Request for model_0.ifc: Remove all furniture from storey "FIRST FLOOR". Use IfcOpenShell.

First a look at what the model holds.

```python
import ifcopenshell
import ifcopenshell.util.element

model = ifcopenshell.open("model_0.ifc")
print(model.schema)
storey = next(s for s in model.by_type("IfcBuildingStorey") if s.Name == "FIRST FLOOR")
furniture = [e for e in ifcopenshell.util.element.get_decomposition(storey) if e.is_a("IfcFurnishingElement")]
seen = {}
for e in furniture:
    element_type = ifcopenshell.util.element.get_type(e)
    name = element_type.Name if element_type not in (None, e) else None
    seen[name] = seen.get(name, 0) + 1
for name, count in sorted(seen.items(), key=str):
    print(count, "x", name)
```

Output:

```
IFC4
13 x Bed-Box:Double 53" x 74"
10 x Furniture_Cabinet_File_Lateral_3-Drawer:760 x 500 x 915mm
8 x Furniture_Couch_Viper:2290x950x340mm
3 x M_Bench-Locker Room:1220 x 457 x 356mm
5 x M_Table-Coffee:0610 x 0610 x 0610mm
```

```python
import ifcopenshell
import ifcopenshell.api.root
import ifcopenshell.util.element

model = ifcopenshell.open("model_0.ifc")

storey = next(s for s in model.by_type("IfcBuildingStorey") if s.Name == "FIRST FLOOR")
furniture = [e for e in ifcopenshell.util.element.get_decomposition(storey) if e.is_a("IfcFurnishingElement")]

for e in furniture:
    ifcopenshell.api.root.remove_product(model, product=e)
print(len(furniture), "removed")

model.write("model_0_edited.ifc")
```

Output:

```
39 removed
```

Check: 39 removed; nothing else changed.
